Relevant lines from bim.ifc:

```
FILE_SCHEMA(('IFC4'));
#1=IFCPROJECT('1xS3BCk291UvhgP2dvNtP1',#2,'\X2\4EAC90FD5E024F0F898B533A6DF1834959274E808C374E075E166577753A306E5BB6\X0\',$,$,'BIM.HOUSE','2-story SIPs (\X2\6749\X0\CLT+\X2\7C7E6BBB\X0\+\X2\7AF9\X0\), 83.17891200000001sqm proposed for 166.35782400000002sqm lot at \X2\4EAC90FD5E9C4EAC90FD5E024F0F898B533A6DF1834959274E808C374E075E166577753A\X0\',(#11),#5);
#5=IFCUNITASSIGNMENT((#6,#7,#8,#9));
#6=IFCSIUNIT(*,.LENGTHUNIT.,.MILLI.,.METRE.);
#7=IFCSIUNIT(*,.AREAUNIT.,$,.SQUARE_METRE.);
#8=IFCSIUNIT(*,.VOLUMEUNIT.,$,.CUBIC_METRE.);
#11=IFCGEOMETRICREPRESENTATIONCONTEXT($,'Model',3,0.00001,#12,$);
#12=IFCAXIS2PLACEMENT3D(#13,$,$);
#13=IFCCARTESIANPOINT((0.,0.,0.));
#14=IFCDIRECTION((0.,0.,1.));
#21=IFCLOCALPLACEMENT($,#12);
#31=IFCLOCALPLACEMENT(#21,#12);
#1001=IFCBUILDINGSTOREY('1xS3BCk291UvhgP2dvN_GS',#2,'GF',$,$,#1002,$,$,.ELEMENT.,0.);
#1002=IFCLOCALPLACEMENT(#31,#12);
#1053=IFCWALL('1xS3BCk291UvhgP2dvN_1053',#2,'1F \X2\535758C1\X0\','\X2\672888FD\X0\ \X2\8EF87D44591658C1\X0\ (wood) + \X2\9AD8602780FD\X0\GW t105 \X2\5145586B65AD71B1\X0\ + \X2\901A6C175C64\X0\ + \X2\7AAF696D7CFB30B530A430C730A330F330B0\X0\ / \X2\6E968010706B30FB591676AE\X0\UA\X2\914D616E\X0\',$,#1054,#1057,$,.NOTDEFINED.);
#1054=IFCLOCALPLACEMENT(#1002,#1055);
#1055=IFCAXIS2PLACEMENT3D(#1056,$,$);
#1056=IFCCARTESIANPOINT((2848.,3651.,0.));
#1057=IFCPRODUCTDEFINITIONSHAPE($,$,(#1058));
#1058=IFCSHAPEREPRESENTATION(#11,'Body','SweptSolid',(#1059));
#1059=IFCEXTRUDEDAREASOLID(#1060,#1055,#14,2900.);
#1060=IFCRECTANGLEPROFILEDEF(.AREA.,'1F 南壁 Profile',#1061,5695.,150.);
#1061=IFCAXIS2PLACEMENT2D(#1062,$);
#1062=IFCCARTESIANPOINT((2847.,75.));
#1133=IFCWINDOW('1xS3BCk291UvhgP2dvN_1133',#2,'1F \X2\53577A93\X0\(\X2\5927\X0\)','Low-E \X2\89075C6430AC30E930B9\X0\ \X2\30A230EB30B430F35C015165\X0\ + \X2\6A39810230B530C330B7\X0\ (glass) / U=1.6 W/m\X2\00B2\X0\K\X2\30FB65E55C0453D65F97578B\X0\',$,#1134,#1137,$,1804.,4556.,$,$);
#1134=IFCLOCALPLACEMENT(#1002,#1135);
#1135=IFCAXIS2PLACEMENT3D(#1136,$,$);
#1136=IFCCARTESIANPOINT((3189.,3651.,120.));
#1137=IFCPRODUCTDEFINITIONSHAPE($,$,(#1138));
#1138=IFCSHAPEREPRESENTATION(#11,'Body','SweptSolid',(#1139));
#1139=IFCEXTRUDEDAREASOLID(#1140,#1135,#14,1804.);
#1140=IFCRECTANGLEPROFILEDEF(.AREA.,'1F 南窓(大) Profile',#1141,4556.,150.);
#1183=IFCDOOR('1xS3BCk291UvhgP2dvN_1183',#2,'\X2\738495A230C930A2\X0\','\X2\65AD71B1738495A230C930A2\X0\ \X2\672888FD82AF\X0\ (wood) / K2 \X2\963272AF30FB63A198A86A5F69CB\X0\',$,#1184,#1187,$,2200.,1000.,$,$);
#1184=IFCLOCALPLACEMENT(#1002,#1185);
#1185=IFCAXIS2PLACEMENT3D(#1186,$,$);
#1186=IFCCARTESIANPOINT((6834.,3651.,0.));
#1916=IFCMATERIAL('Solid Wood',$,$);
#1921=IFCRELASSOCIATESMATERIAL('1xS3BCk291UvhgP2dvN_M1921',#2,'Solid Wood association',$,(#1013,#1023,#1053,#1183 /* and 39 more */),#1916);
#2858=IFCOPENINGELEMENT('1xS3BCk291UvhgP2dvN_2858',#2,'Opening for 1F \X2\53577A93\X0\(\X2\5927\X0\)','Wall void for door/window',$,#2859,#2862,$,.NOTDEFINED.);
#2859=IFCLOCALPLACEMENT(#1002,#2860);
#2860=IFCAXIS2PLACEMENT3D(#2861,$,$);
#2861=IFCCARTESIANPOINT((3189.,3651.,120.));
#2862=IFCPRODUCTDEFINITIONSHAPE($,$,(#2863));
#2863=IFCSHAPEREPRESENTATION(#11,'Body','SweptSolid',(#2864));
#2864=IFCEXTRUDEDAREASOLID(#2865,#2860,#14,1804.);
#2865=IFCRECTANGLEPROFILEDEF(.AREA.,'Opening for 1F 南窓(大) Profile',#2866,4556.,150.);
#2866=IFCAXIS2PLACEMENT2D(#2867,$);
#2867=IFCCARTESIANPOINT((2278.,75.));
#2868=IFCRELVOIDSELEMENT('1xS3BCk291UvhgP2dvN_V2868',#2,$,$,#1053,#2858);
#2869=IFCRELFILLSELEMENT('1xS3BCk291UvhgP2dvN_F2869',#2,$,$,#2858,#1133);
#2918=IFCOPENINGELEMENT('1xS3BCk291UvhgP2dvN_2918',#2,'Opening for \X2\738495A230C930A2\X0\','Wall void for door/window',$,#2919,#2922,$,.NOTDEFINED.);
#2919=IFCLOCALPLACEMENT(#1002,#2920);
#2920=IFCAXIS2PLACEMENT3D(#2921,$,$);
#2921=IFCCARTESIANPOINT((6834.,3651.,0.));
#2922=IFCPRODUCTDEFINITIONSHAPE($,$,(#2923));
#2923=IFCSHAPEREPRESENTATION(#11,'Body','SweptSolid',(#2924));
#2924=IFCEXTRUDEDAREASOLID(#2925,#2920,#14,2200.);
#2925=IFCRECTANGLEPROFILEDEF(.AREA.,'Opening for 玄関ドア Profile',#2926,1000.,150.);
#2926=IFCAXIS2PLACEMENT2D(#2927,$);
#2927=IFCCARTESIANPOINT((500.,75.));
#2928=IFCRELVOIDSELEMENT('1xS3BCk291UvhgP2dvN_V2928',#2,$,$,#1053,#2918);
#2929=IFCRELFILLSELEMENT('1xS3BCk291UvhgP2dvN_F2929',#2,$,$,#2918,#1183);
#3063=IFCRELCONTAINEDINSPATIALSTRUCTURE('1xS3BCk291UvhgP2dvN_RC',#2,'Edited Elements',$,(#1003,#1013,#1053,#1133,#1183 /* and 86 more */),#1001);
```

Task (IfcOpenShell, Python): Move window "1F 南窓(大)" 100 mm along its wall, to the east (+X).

```python
import ifcopenshell
import ifcopenshell.api.geometry
import ifcopenshell.util.placement

model = ifcopenshell.open("bim.ifc")

window = model.by_id(1133)
opening = window.FillsVoids[0].RelatingOpeningElement
wall = opening.VoidsElements[0].RelatingBuildingElement

wall_matrix = ifcopenshell.util.placement.get_local_placement(wall.ObjectPlacement)
shift = wall_matrix[:3, 0] * 100.0
before = ifcopenshell.util.placement.get_local_placement(window.ObjectPlacement)[:3, 3].copy()

# The window is not placed relative to its opening, so move both.
for product in (opening, window):
    matrix = ifcopenshell.util.placement.get_local_placement(product.ObjectPlacement)
    matrix[:3, 3] += shift
    ifcopenshell.api.geometry.edit_object_placement(model, product=product, matrix=matrix, is_si=False)

after = ifcopenshell.util.placement.get_local_placement(window.ObjectPlacement)[:3, 3]
print("window moved by", (after - before).round(3) + 0.0)

model.write("bim_updated.ifc")
```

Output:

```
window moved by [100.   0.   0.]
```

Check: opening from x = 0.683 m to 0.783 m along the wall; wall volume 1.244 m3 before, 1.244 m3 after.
